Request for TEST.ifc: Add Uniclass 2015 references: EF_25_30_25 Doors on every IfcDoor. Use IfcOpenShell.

First a look at what the model holds.

```python
import ifcopenshell

model = ifcopenshell.open("TEST.ifc")
print(model.schema)
print("classifications:", [c.Name for c in model.by_type("IfcClassification")])
for ifc_class in ("IfcDoor", "IfcRoof", "IfcStair", "IfcWall", "IfcWindow"):
    print(ifc_class, len(model.by_type(ifc_class)))
```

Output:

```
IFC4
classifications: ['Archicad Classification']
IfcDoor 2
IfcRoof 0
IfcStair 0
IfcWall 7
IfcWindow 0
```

```python
import ifcopenshell
import ifcopenshell.api.classification

model = ifcopenshell.open("TEST.ifc")

system = ifcopenshell.api.classification.add_classification(model, classification="Uniclass 2015")

codes = {
    "IfcDoor": ("EF_25_30_25", "Doors"),
}
for ifc_class, (code, name) in codes.items():
    products = model.by_type(ifc_class)
    ifcopenshell.api.classification.add_reference(
        model, products=products, classification=system, identification=code, name=name
    )
    print(code, len(products))

model.write("TEST-out.ifc")
```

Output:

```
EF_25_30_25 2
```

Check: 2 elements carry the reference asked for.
